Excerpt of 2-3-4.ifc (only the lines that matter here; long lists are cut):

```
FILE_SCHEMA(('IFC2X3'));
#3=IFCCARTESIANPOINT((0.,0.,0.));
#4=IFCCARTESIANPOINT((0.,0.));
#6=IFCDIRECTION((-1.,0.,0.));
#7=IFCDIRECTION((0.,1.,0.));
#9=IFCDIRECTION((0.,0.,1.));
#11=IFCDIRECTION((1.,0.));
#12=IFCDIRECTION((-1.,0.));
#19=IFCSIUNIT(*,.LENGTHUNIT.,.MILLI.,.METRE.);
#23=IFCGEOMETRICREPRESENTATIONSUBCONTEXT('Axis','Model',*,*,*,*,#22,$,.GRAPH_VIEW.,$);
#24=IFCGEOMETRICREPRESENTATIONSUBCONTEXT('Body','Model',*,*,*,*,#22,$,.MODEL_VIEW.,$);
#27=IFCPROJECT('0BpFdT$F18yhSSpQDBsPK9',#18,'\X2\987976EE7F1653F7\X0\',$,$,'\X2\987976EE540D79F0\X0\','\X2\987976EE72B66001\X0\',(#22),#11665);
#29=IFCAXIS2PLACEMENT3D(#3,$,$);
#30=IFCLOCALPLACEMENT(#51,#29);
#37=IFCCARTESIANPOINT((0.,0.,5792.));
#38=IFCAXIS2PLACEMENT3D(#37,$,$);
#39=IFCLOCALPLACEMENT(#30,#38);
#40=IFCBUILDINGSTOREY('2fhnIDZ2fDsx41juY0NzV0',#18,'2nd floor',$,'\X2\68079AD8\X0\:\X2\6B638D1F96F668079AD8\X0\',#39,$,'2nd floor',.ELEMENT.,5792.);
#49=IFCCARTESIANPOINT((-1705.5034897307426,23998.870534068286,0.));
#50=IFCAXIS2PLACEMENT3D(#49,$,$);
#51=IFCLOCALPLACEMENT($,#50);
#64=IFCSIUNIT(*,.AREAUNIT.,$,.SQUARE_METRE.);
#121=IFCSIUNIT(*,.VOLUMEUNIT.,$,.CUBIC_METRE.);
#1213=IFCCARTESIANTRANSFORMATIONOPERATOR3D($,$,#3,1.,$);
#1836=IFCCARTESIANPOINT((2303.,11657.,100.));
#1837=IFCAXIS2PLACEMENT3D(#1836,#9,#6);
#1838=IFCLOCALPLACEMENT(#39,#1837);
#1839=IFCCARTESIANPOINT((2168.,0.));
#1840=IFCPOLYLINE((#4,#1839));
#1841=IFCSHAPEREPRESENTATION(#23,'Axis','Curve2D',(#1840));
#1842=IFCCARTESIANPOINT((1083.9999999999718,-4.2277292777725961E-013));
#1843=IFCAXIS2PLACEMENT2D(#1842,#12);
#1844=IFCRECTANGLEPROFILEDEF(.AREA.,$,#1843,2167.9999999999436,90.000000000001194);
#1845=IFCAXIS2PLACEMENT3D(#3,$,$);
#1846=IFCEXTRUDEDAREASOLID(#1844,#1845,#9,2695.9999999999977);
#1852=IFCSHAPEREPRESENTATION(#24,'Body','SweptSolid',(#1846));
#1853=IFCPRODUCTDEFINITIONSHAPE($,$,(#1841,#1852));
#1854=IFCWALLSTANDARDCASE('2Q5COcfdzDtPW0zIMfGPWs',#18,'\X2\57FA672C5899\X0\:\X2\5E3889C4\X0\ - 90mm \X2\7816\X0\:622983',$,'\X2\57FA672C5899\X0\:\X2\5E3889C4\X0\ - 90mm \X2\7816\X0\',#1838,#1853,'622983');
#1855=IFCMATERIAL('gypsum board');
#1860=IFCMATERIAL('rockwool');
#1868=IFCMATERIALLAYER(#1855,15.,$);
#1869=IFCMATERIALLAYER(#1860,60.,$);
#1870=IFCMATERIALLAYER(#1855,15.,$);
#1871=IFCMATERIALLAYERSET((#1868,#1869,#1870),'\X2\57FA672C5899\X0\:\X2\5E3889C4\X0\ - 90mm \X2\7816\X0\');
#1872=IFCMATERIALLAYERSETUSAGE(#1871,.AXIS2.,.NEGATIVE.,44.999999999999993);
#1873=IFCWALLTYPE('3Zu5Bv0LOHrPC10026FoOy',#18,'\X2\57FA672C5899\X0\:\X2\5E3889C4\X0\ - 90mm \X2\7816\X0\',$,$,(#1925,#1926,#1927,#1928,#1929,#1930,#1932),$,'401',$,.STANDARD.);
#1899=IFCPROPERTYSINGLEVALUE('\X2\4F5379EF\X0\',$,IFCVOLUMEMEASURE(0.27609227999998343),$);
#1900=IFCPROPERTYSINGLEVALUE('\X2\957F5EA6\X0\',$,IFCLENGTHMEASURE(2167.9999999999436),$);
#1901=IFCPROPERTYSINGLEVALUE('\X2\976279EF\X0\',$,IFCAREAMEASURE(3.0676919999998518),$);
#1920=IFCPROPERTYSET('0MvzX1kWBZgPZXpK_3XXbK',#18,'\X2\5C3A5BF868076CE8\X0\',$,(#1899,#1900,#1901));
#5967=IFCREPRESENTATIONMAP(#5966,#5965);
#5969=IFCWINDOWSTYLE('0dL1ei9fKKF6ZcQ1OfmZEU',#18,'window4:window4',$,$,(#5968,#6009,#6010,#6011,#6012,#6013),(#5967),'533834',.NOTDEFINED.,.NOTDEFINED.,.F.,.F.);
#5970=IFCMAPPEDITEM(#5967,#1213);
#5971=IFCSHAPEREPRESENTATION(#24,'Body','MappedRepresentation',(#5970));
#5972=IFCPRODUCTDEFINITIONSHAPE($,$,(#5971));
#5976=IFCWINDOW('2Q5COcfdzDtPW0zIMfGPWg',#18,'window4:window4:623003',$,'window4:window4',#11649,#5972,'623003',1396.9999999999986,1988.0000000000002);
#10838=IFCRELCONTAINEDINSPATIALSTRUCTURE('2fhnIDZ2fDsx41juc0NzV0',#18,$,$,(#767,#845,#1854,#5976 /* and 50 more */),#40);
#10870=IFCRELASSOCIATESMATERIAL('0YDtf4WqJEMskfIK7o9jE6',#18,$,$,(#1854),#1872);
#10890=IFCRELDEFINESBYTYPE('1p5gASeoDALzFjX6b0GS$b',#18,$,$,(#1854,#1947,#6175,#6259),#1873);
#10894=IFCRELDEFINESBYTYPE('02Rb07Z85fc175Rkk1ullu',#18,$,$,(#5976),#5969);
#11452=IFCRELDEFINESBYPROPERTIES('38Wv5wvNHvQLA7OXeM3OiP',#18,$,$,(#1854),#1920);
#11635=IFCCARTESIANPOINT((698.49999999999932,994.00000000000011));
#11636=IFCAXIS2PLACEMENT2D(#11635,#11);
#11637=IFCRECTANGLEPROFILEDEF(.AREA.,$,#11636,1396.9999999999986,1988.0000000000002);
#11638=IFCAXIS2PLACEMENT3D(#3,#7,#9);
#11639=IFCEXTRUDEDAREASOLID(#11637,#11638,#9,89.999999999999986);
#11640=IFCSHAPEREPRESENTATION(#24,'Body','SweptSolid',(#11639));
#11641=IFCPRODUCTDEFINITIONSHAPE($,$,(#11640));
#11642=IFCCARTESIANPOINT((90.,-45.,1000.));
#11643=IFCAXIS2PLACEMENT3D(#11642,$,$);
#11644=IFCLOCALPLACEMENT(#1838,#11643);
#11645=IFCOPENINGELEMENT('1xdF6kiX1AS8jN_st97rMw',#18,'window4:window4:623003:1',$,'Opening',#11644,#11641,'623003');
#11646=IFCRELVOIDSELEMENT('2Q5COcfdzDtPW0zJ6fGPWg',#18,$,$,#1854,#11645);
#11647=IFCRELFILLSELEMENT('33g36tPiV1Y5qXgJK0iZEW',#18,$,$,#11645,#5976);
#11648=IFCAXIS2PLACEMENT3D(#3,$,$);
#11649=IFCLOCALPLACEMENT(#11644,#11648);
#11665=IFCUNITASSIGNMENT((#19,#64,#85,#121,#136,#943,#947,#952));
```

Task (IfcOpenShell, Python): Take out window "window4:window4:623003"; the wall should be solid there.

```python
import ifcopenshell
import ifcopenshell.api.feature
import ifcopenshell.api.pset
import ifcopenshell.api.root
import ifcopenshell.geom
import ifcopenshell.util.element
import ifcopenshell.util.shape
import ifcopenshell.util.unit

model = ifcopenshell.open("2-3-4.ifc")
area_scale = ifcopenshell.util.unit.calculate_unit_scale(model, "AREAUNIT")
volume_scale = ifcopenshell.util.unit.calculate_unit_scale(model, "VOLUMEUNIT")
settings = ifcopenshell.geom.settings()


def volume(element):
    """Net volume in cubic metres, openings subtracted."""
    shape = ifcopenshell.geom.create_shape(settings, element)
    return ifcopenshell.util.shape.get_volume(shape.geometry)


window = model.by_guid("2Q5COcfdzDtPW0zIMfGPWg")
opening = window.FillsVoids[0].RelatingOpeningElement
wall = opening.VoidsElements[0].RelatingBuildingElement
before = volume(wall)

ifcopenshell.api.root.remove_product(model, product=window)
ifcopenshell.api.feature.remove_feature(model, feature=opening)

after = volume(wall)
thickness = 0.09  # wall thickness in metres

# Update the wall's stored quantities.
pset = model.by_id(ifcopenshell.util.element.get_pset(wall, "尺寸标注", should_inherit=False)["id"])
ifcopenshell.api.pset.edit_pset(model, pset=pset, properties={
    "体积": model.create_entity("IfcVolumeMeasure", after / volume_scale),
    "面积": model.create_entity("IfcAreaMeasure", after / thickness / area_scale),
})

print(f"wall volume {before:.3f} -> {after:.3f} m3")

model.write("2-3-4_rev.ifc")
```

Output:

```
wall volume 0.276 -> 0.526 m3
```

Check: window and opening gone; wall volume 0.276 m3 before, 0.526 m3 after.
